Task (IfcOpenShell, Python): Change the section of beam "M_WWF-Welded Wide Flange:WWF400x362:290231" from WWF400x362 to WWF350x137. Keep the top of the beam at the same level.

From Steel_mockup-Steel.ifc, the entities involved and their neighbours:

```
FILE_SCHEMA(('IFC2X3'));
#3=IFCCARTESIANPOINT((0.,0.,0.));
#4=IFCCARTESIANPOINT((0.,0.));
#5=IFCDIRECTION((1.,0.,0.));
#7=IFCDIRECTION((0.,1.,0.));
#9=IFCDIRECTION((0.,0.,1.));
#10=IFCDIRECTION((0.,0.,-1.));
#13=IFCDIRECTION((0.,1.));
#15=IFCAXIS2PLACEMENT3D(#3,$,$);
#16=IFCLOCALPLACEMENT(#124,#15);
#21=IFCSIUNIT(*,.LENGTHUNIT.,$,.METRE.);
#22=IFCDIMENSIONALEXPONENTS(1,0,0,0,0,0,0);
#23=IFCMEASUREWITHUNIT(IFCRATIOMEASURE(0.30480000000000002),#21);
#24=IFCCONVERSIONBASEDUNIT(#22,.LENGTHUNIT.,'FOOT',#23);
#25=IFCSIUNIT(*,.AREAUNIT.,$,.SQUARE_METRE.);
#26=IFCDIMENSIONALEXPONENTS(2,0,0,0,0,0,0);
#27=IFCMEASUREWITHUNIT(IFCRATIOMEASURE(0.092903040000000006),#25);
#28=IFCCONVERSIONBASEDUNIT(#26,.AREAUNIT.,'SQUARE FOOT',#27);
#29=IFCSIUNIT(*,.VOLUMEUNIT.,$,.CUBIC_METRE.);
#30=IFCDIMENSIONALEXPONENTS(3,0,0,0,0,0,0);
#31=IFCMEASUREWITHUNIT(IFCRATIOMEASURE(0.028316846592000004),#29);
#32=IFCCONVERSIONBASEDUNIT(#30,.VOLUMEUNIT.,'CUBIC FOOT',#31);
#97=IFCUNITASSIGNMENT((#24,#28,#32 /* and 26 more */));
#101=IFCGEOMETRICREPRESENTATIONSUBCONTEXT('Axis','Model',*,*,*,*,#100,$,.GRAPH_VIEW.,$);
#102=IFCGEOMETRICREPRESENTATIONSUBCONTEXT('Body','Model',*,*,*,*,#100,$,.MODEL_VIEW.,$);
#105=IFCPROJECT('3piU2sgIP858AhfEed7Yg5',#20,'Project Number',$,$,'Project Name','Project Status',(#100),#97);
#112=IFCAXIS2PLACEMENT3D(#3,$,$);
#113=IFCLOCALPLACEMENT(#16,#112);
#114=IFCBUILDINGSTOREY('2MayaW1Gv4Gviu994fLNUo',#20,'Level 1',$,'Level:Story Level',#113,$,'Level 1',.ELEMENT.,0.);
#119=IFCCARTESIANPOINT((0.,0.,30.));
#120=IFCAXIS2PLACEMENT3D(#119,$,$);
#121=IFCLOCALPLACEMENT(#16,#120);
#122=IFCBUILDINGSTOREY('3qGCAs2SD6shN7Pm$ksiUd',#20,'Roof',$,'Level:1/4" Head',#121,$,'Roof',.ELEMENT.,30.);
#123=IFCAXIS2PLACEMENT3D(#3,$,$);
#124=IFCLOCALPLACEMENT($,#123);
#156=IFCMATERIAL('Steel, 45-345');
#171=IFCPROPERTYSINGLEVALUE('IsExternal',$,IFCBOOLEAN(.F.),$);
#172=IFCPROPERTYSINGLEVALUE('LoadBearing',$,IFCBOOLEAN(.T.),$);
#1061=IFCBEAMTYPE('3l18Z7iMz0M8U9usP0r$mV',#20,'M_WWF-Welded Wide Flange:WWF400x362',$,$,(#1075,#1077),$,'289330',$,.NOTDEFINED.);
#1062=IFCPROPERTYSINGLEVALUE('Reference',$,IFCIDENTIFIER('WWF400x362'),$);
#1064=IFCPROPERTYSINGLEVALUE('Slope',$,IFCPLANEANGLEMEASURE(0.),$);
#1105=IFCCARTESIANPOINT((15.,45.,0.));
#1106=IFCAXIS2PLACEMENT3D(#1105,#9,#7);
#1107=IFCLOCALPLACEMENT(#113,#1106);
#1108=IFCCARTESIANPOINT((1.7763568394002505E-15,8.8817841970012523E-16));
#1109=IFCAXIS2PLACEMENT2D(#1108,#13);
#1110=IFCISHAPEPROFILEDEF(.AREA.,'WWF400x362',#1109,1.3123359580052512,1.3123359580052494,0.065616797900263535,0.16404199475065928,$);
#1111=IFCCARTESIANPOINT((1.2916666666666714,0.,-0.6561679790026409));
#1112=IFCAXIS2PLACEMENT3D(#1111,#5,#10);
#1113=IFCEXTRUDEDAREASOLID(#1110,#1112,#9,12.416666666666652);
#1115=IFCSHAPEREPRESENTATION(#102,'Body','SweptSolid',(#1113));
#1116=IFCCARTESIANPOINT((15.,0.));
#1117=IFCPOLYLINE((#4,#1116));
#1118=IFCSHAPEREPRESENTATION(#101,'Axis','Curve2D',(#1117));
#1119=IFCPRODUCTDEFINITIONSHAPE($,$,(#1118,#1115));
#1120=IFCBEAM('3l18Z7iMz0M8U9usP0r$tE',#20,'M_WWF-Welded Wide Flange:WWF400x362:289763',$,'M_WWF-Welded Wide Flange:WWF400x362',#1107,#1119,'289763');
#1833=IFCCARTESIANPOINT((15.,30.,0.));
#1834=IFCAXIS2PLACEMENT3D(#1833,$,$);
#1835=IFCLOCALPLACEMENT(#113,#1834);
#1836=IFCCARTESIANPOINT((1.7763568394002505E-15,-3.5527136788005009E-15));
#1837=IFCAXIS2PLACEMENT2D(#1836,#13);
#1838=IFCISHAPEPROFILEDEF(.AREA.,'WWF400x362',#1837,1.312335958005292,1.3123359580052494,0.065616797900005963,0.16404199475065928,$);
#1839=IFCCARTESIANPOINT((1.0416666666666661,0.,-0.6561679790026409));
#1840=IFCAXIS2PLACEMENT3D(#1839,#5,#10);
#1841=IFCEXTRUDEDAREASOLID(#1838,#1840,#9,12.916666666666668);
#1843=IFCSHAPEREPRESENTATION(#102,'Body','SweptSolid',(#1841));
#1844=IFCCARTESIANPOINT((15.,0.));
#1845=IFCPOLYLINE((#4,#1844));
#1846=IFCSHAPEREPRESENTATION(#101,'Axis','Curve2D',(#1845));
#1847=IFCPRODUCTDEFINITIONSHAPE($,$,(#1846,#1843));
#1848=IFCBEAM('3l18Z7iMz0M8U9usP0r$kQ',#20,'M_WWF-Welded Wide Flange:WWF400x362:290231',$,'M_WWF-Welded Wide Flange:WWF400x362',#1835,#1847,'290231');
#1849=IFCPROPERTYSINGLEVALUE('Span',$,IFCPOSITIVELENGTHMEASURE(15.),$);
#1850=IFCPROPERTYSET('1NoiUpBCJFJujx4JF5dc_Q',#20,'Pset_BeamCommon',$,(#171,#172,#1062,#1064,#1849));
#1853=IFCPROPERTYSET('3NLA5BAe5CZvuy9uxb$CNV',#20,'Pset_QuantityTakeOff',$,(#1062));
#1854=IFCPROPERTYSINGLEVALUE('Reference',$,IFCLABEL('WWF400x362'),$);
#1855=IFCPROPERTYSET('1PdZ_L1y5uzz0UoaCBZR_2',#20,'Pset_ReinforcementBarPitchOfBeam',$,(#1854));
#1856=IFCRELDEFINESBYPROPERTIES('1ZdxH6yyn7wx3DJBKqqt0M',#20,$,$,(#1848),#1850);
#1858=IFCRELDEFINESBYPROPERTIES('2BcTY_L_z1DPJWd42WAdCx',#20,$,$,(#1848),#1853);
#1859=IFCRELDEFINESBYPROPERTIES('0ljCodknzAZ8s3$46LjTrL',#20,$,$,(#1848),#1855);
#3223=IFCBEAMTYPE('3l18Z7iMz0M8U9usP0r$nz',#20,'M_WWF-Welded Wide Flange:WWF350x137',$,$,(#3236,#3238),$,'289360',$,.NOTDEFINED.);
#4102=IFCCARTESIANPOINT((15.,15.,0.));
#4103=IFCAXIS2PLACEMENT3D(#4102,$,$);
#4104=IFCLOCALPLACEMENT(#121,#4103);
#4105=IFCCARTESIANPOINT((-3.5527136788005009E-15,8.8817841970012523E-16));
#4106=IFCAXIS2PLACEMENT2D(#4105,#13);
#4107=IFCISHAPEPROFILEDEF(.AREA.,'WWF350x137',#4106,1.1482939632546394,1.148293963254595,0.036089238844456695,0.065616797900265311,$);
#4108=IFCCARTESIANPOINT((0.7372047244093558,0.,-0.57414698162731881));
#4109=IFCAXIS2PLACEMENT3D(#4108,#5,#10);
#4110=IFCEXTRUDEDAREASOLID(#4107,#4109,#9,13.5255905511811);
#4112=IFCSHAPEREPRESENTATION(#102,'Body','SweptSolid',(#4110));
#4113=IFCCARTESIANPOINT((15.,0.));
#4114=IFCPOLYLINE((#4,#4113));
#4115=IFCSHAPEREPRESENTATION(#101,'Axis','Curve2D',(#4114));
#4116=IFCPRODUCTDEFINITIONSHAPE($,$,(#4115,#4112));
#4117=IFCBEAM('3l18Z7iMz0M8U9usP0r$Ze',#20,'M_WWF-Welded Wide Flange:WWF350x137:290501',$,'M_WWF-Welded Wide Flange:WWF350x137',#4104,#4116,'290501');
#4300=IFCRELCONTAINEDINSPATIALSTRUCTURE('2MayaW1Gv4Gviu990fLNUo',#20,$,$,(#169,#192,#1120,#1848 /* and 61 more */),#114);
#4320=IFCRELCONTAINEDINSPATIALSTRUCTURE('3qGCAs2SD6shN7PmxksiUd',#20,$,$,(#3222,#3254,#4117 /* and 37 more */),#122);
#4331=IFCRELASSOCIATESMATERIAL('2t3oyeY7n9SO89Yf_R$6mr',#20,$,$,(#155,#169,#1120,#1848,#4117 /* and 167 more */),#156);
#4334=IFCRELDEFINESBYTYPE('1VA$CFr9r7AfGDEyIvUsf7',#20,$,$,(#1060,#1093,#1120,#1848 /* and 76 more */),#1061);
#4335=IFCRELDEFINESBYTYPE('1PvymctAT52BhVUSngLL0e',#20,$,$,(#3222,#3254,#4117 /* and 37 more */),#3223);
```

```python
import ifcopenshell
import ifcopenshell.api.pset
import ifcopenshell.api.type
import ifcopenshell.util.element
import ifcopenshell.util.representation

model = ifcopenshell.open("Steel_mockup-Steel.ifc")

member = model.by_guid("3l18Z7iMz0M8U9usP0r$kQ")
source = next(p for p in model.by_type("IfcIShapeProfileDef") if p.ProfileName == "WWF350x137")

body = ifcopenshell.util.representation.get_representation(member, "Model", "Body")
solid = body.Items[0]
old_profile = solid.SweptArea

# Copy the section's sizes but keep this member's own profile position.
profile = ifcopenshell.util.element.copy(model, source)
# Profiles are centred, so shift by half the change in depth to hold the top.
shift = (old_profile.OverallDepth - profile.OverallDepth) / 2
x, y = old_profile.Position.Location.Coordinates
up = (-1.0, 0.0)  # upwards, in the solid's own plane
location = model.createIfcCartesianPoint((x + up[0] * shift, y + up[1] * shift))
profile.Position = model.createIfcAxis2Placement2D(location, old_profile.Position.RefDirection)
solid.SweptArea = profile
if not model.get_total_inverses(old_profile):
    ifcopenshell.util.element.remove_deep2(model, old_profile)

new_type = model.by_id(3223)
ifcopenshell.api.type.assign_type(
    model, related_objects=[member], relating_type=new_type, should_map_representations=False
)
member.Name = member.Name.replace("WWF400x362", "WWF350x137")
member.ObjectType = "M_WWF-Welded Wide Flange:WWF350x137"
pset = model.by_id(ifcopenshell.util.element.get_pset(member, "Pset_BeamCommon", should_inherit=False)["id"])
ifcopenshell.api.pset.edit_pset(model, pset=pset, properties={"Reference": "WWF350x137"})
pset = model.by_id(ifcopenshell.util.element.get_pset(member, "Pset_QuantityTakeOff", should_inherit=False)["id"])
ifcopenshell.api.pset.edit_pset(model, pset=pset, properties={"Reference": "WWF350x137"})
pset = model.by_id(ifcopenshell.util.element.get_pset(member, "Pset_ReinforcementBarPitchOfBeam", should_inherit=False)["id"])
ifcopenshell.api.pset.edit_pset(model, pset=pset, properties={"Reference": "WWF350x137"})

print(solid.SweptArea)

model.write("Steel_mockup-Steel_v2.ifc")
```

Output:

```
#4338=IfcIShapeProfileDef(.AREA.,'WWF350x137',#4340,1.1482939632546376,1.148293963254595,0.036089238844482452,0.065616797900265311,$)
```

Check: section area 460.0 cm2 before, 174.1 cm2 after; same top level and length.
